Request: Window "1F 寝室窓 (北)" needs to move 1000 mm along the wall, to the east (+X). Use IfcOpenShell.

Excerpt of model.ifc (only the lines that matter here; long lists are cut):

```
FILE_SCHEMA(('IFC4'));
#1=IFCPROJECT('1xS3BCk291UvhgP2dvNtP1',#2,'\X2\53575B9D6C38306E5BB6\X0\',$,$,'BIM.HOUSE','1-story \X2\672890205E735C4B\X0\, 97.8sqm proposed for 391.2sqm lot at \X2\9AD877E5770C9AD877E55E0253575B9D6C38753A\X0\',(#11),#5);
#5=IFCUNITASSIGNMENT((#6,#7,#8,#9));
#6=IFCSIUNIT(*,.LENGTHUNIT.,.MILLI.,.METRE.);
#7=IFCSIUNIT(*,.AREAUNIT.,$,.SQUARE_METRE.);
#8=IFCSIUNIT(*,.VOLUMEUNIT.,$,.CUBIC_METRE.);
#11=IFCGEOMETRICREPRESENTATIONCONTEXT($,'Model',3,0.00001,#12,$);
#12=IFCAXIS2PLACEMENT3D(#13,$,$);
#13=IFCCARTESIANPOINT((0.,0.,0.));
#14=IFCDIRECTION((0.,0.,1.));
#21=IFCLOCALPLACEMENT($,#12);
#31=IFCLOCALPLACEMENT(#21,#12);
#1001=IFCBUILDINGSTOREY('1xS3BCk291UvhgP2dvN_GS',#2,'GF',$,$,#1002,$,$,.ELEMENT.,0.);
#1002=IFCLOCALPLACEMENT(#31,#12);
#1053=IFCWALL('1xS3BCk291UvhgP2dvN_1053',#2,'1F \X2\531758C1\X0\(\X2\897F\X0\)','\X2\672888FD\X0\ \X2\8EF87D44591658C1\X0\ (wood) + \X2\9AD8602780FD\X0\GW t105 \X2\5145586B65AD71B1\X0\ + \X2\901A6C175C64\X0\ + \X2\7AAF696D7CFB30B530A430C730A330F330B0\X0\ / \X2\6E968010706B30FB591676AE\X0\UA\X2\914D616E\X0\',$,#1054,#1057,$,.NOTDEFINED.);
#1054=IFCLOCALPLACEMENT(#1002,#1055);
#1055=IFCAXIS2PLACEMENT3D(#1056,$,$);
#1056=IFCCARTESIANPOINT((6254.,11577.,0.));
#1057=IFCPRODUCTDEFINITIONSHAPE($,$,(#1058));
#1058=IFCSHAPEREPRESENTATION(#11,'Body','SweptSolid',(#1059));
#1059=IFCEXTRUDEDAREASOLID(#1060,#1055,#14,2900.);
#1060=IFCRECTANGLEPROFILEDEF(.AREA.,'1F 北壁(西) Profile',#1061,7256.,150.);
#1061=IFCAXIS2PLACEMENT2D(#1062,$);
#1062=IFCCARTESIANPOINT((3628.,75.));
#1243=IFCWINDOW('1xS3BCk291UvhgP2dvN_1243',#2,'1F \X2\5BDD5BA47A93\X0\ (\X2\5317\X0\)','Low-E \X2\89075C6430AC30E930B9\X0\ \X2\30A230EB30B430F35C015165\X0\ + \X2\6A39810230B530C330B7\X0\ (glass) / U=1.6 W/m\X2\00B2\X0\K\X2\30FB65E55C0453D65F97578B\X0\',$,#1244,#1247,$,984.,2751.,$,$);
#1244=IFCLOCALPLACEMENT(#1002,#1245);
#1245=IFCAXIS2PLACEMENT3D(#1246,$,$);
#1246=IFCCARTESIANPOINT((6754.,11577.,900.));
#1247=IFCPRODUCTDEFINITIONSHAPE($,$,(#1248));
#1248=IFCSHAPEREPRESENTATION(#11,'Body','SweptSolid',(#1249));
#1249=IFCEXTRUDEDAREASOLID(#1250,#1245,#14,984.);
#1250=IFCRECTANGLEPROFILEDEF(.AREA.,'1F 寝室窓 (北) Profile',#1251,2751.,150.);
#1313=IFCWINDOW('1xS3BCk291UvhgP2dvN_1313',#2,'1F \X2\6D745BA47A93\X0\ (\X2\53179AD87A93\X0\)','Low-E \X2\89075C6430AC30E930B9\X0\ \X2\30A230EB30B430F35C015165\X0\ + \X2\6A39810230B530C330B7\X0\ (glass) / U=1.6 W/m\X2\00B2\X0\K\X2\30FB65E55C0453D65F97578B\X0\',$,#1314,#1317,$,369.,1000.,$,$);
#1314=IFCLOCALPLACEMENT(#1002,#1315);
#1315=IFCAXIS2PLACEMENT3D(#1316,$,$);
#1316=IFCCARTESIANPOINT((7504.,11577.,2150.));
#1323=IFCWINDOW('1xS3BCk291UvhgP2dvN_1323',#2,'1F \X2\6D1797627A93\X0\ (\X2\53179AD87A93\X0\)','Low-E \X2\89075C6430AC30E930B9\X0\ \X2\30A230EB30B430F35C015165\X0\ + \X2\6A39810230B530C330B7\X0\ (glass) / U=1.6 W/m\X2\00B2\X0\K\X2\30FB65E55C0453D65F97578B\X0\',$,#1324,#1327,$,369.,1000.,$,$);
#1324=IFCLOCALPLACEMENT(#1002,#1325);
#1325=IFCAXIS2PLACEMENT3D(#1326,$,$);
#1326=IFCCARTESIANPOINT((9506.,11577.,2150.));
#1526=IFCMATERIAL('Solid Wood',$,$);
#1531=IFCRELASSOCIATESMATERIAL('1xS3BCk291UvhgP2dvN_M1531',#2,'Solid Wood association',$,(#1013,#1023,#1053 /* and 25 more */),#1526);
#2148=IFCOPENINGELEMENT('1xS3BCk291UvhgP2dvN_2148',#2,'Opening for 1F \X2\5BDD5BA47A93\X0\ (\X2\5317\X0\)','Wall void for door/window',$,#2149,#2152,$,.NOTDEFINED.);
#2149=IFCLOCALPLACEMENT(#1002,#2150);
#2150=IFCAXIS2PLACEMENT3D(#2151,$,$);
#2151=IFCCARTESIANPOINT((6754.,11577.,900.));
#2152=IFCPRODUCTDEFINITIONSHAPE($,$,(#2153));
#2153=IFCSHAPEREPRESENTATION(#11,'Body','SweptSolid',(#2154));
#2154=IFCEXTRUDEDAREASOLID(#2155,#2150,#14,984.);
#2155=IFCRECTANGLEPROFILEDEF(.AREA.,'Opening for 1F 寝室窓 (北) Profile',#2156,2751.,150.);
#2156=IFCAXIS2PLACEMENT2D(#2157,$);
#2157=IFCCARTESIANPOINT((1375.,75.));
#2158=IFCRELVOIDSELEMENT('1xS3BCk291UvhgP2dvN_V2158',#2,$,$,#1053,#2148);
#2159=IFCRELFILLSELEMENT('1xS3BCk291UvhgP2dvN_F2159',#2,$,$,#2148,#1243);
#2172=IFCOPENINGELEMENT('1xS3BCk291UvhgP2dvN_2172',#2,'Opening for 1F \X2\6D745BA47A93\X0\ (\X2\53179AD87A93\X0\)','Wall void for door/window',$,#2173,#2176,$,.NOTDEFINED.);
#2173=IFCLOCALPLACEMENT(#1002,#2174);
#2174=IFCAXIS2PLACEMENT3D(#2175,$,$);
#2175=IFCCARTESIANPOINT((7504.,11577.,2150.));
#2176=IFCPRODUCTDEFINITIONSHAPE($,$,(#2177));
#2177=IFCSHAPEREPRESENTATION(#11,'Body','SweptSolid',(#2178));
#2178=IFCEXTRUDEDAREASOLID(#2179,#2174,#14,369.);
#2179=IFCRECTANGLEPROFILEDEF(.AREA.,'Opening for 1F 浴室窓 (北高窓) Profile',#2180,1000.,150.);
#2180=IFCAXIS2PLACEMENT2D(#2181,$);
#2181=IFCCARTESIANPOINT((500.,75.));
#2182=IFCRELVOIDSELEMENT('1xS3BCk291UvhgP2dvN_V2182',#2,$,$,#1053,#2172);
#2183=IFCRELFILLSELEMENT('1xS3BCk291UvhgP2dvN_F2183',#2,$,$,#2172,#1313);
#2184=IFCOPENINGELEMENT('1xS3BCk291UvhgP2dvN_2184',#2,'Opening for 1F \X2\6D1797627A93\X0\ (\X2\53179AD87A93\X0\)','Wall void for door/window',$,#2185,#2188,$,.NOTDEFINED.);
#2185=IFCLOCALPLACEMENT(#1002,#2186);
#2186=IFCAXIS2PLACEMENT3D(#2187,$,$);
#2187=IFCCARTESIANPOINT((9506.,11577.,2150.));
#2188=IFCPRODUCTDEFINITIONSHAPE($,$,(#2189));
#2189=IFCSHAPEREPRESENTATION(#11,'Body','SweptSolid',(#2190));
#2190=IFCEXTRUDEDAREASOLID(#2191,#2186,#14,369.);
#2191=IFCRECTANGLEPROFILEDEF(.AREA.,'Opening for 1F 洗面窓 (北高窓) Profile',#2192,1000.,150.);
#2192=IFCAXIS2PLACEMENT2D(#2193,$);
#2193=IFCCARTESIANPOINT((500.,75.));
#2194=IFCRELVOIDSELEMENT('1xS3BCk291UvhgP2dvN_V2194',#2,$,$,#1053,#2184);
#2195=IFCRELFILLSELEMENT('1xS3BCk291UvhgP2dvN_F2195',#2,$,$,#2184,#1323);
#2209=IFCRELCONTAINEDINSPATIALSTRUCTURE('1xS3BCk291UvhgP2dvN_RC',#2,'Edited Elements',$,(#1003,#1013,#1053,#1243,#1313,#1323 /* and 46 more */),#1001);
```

```python
import ifcopenshell
import ifcopenshell.api.geometry
import ifcopenshell.util.placement

model = ifcopenshell.open("model.ifc")

window = model.by_guid("1xS3BCk291UvhgP2dvN_1243")
opening = window.FillsVoids[0].RelatingOpeningElement
wall = opening.VoidsElements[0].RelatingBuildingElement

wall_matrix = ifcopenshell.util.placement.get_local_placement(wall.ObjectPlacement)
shift = wall_matrix[:3, 0] * 1000.0
before = ifcopenshell.util.placement.get_local_placement(window.ObjectPlacement)[:3, 3].copy()

# The window is not placed relative to its opening, so move both.
for product in (opening, window):
    matrix = ifcopenshell.util.placement.get_local_placement(product.ObjectPlacement)
    matrix[:3, 3] += shift
    ifcopenshell.api.geometry.edit_object_placement(model, product=product, matrix=matrix, is_si=False)

after = ifcopenshell.util.placement.get_local_placement(window.ObjectPlacement)[:3, 3]
print("window moved by", (after - before).round(3) + 0.0)

model.write("model-out.ifc")
```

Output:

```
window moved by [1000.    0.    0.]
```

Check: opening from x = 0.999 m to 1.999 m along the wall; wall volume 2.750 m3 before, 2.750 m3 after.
